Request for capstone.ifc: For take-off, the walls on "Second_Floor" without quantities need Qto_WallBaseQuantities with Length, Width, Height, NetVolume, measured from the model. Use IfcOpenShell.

First a look at what the model holds.

```python
import ifcopenshell
import ifcopenshell.util.element
import ifcopenshell.util.unit

model = ifcopenshell.open("capstone.ifc")
print(model.schema)
for unit_type in ("LENGTHUNIT", "AREAUNIT", "VOLUMEUNIT"):
    print(unit_type, ifcopenshell.util.unit.calculate_unit_scale(model, unit_type))
storey = next(s for s in model.by_type("IfcBuildingStorey") if s.Name == "Second_Floor")
walls = [e for e in ifcopenshell.util.element.get_decomposition(storey) if e.is_a("IfcWall")]
for e in sorted(walls, key=lambda e: e.id()):
    print(e.id(), e.is_a(), e.Name, list(ifcopenshell.util.element.get_psets(e, qtos_only=True)), sep=" | ")
```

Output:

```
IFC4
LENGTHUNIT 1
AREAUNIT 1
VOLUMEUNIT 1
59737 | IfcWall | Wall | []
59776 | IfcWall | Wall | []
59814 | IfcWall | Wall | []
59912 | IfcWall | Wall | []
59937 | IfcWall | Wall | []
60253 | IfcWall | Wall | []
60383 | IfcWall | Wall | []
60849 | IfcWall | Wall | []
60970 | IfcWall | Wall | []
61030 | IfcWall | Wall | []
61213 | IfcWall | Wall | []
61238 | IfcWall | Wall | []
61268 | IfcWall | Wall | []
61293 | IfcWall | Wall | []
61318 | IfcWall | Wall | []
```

```python
import ifcopenshell
import ifcopenshell.api.pset
import ifcopenshell.geom
import ifcopenshell.util.element
import ifcopenshell.util.shape
import ifcopenshell.util.unit

model = ifcopenshell.open("capstone.ifc")
unit_scale = ifcopenshell.util.unit.calculate_unit_scale(model)
volume_scale = ifcopenshell.util.unit.calculate_unit_scale(model, "VOLUMEUNIT")
settings = ifcopenshell.geom.settings()

storey = next(s for s in model.by_type("IfcBuildingStorey") if s.Name == "Second_Floor")
walls = [e for e in ifcopenshell.util.element.get_decomposition(storey) if e.is_a("IfcWall")]

for e in sorted(walls, key=lambda e: e.id()):
    if ifcopenshell.util.element.get_psets(e, qtos_only=True, should_inherit=False):
        continue
    # Geometry comes back in metres, in the element's own axes.
    shape = ifcopenshell.geom.create_shape(settings, e)
    values = {
        "Length": ifcopenshell.util.shape.get_x(shape.geometry) / unit_scale,
        "Width": ifcopenshell.util.shape.get_y(shape.geometry) / unit_scale,
        "Height": ifcopenshell.util.shape.get_z(shape.geometry) / unit_scale,
        "NetVolume": ifcopenshell.util.shape.get_volume(shape.geometry) / volume_scale,
    }
    qto = ifcopenshell.api.pset.add_qto(model, product=e, name="Qto_WallBaseQuantities")
    ifcopenshell.api.pset.edit_qto(model, qto=qto, properties=values)
    print(e.id(), {k: round(v, 3) for k, v in values.items()})

model.write("capstone_edited.ifc")
```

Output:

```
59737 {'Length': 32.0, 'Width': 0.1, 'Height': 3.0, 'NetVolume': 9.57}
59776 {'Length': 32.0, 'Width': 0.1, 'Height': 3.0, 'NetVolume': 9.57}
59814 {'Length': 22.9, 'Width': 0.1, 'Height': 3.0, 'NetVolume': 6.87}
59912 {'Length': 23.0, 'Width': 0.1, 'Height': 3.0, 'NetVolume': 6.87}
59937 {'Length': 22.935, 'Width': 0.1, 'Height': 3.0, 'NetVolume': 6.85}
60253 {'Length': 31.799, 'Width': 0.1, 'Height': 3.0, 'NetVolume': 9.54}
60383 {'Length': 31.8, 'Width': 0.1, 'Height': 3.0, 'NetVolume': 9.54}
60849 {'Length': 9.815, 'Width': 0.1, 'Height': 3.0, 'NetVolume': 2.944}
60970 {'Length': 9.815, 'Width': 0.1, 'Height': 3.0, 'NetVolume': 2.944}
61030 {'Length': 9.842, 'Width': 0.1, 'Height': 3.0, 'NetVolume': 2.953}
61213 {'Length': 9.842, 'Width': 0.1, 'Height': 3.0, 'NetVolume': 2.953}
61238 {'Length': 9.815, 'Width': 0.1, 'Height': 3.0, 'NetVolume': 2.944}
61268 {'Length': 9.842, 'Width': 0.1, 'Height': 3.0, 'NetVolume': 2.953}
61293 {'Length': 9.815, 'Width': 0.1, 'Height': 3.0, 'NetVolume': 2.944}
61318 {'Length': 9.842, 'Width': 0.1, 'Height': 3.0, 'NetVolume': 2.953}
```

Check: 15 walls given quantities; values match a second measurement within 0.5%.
